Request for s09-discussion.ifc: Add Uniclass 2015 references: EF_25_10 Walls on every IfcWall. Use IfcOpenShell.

First a look at what the model holds.

```python
import ifcopenshell

model = ifcopenshell.open("s09-discussion.ifc")
print(model.schema)
print("classifications:", [c.Name for c in model.by_type("IfcClassification")])
for ifc_class in ("IfcDoor", "IfcRoof", "IfcStair", "IfcWall", "IfcWindow"):
    print(ifc_class, len(model.by_type(ifc_class)))
```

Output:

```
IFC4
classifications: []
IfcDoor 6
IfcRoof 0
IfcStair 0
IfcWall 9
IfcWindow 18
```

```python
import ifcopenshell
import ifcopenshell.api.classification

model = ifcopenshell.open("s09-discussion.ifc")

system = ifcopenshell.api.classification.add_classification(model, classification="Uniclass 2015")

codes = {
    "IfcWall": ("EF_25_10", "Walls"),
}
for ifc_class, (code, name) in codes.items():
    products = model.by_type(ifc_class)
    ifcopenshell.api.classification.add_reference(
        model, products=products, classification=system, identification=code, name=name
    )
    print(code, len(products))

model.write("s09-discussion_rev.ifc")
```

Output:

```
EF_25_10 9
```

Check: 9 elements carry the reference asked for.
